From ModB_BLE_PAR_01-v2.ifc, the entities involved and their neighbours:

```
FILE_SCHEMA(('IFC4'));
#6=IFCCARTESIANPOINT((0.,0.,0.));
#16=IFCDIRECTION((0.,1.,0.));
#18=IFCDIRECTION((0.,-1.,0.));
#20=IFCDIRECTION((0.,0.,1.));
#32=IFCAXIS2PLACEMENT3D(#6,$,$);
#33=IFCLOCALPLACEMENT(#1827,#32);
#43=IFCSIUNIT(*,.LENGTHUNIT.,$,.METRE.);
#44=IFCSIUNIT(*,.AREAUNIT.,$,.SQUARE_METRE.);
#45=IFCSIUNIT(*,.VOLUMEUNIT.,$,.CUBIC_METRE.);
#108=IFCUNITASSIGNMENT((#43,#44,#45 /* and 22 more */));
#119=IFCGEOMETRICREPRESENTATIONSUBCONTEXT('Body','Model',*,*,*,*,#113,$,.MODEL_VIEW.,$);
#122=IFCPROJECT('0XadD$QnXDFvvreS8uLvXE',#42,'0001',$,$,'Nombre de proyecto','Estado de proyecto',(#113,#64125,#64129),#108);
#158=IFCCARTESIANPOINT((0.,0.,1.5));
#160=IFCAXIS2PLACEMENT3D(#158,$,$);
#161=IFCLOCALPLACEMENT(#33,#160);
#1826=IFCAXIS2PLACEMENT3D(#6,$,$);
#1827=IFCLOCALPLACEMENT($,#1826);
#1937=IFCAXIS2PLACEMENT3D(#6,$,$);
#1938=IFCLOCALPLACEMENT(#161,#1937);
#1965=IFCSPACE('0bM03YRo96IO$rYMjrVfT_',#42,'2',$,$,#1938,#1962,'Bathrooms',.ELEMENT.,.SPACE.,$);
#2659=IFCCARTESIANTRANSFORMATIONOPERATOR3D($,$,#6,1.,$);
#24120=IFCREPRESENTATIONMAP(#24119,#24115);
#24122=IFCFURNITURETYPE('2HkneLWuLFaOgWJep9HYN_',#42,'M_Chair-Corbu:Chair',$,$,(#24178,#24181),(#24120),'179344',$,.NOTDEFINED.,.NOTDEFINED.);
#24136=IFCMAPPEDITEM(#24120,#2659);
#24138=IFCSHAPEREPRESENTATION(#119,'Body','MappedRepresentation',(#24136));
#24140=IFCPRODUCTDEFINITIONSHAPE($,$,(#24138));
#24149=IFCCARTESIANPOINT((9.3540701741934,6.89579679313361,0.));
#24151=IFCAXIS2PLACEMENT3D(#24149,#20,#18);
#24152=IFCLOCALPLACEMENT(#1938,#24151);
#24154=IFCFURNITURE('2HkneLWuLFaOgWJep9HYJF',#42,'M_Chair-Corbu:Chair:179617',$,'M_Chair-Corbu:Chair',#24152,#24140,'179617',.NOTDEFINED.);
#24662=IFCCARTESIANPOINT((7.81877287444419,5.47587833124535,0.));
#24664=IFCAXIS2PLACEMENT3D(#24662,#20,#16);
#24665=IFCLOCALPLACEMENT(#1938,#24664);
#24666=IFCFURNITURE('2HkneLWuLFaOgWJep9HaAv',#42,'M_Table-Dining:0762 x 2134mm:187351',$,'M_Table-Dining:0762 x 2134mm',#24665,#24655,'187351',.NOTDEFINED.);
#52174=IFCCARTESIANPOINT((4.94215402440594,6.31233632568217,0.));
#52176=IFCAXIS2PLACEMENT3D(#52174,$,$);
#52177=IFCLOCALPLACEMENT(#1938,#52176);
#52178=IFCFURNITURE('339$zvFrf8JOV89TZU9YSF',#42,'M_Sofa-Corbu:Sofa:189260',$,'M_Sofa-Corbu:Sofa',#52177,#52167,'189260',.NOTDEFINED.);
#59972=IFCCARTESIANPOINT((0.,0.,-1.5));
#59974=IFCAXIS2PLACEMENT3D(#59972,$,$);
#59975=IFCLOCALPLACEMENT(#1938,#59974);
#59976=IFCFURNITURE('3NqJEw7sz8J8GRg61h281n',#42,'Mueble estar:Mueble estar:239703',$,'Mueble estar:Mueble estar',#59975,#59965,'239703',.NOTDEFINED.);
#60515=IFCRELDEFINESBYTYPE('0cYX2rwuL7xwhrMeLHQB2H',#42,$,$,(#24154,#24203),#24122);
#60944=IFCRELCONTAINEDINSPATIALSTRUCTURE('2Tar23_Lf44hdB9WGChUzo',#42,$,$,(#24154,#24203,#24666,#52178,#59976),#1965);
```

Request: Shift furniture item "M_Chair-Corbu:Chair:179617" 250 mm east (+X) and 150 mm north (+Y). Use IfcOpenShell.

```python
import ifcopenshell
import ifcopenshell.api.geometry
import ifcopenshell.util.placement

model = ifcopenshell.open("ModB_BLE_PAR_01-v2.ifc")

item = model.by_guid("2HkneLWuLFaOgWJep9HYJF")
matrix = ifcopenshell.util.placement.get_local_placement(item.ObjectPlacement)
matrix[0, 3] += 0.25
matrix[1, 3] += 0.15
ifcopenshell.api.geometry.edit_object_placement(model, product=item, matrix=matrix, is_si=False)

print(ifcopenshell.util.placement.get_local_placement(item.ObjectPlacement).round(3) + 0.0)

model.write("ModB_BLE_PAR_01-v2_rev.ifc")
```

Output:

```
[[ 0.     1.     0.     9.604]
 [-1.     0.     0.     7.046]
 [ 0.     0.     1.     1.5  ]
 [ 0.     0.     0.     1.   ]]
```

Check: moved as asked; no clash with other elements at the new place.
